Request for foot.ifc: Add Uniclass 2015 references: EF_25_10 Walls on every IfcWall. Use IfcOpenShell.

First a look at what the model holds.

```python
import ifcopenshell

model = ifcopenshell.open("foot.ifc")
print(model.schema)
print("classifications:", [c.Name for c in model.by_type("IfcClassification")])
for ifc_class in ("IfcDoor", "IfcRoof", "IfcStair", "IfcWall", "IfcWindow"):
    print(ifc_class, len(model.by_type(ifc_class)))
```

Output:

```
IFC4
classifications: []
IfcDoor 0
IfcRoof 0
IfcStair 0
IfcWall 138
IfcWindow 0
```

```python
import ifcopenshell
import ifcopenshell.api.classification

model = ifcopenshell.open("foot.ifc")

system = ifcopenshell.api.classification.add_classification(model, classification="Uniclass 2015")

codes = {
    "IfcWall": ("EF_25_10", "Walls"),
}
for ifc_class, (code, name) in codes.items():
    products = model.by_type(ifc_class)
    ifcopenshell.api.classification.add_reference(
        model, products=products, classification=system, identification=code, name=name
    )
    print(code, len(products))

model.write("foot_edited.ifc")
```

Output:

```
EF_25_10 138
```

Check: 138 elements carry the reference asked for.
